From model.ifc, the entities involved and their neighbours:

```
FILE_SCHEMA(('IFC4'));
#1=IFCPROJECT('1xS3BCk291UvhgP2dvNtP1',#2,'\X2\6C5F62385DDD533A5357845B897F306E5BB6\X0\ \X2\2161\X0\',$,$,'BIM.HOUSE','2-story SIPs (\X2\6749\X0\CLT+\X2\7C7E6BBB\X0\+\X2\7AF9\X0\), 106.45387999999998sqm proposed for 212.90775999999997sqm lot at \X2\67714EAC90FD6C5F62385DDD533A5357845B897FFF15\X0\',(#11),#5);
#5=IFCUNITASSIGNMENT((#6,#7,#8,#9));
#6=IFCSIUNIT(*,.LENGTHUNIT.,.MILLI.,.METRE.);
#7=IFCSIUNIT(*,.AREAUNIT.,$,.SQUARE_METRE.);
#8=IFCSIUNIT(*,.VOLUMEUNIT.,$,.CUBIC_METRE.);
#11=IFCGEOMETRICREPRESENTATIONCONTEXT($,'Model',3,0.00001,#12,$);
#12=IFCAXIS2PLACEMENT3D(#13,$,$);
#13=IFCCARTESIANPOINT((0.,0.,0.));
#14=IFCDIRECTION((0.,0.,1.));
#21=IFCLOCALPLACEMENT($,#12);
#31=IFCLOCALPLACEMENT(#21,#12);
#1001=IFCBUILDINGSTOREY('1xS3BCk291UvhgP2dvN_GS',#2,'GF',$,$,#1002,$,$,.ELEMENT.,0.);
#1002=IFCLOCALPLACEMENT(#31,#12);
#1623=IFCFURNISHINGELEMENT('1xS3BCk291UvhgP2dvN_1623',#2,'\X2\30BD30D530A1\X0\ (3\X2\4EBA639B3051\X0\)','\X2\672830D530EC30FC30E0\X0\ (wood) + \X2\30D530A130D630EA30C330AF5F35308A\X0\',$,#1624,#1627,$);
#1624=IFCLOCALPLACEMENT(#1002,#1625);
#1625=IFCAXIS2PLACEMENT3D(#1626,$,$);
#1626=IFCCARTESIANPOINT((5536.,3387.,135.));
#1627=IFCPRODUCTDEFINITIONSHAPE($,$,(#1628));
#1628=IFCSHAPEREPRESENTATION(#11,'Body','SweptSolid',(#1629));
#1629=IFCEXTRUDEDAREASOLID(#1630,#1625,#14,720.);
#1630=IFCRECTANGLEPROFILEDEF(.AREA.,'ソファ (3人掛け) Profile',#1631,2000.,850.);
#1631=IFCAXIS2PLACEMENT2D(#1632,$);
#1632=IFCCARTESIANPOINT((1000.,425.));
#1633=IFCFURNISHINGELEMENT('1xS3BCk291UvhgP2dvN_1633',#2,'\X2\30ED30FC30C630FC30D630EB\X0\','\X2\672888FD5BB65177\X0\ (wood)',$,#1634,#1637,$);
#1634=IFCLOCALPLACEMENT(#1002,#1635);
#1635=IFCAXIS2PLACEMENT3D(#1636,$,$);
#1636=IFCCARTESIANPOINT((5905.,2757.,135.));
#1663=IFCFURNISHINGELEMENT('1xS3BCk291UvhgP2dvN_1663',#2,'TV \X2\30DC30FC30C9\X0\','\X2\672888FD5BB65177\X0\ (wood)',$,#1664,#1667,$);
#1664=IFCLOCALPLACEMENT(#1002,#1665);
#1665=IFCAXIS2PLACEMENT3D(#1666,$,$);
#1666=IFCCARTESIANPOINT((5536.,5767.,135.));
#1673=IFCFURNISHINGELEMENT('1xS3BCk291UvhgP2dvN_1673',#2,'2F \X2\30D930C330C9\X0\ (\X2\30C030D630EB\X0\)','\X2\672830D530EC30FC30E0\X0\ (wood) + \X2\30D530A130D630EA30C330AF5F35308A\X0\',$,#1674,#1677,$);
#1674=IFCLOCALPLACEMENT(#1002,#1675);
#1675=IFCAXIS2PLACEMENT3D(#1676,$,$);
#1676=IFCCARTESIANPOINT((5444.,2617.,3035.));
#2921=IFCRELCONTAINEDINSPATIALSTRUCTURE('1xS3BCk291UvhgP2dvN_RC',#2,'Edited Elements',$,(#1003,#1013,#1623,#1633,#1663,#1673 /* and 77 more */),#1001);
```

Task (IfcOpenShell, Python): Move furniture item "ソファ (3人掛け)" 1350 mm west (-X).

```python
import ifcopenshell
import ifcopenshell.api.geometry
import ifcopenshell.util.placement

model = ifcopenshell.open("model.ifc")

item = model.by_guid("1xS3BCk291UvhgP2dvN_1623")
matrix = ifcopenshell.util.placement.get_local_placement(item.ObjectPlacement)
matrix[0, 3] -= 1350.0
ifcopenshell.api.geometry.edit_object_placement(model, product=item, matrix=matrix, is_si=False)

print(ifcopenshell.util.placement.get_local_placement(item.ObjectPlacement).round(3) + 0.0)

model.write("model_edited.ifc")
```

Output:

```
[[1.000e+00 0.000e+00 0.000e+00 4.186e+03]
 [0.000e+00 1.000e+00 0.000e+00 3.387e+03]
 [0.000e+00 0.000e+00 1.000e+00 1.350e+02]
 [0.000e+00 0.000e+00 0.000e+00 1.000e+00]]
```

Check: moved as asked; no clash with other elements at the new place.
